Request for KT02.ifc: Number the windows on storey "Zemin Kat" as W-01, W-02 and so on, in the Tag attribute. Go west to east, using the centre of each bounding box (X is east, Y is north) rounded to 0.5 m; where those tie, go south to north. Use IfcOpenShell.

First a look at what the model holds.

```python
import ifcopenshell
import ifcopenshell.util.element
import ifcopenshell.util.placement

model = ifcopenshell.open("KT02.ifc")
print(model.schema)
storey = next(s for s in model.by_type("IfcBuildingStorey") if s.Name == "Zemin Kat")
windows = [e for e in ifcopenshell.util.element.get_decomposition(storey) if e.is_a("IfcWindow")]
for e in sorted(windows, key=lambda e: e.id()):
    origin = ifcopenshell.util.placement.get_local_placement(e.ObjectPlacement)[:3, 3]
    print(e.id(), e.Tag, e.Name, origin.round(2) + 0.0, sep=" | ")
```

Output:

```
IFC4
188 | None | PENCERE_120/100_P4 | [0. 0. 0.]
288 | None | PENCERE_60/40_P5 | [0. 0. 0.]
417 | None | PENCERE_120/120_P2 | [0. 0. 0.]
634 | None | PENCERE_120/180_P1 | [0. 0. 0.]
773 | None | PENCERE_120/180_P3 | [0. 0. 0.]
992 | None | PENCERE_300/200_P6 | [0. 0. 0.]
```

```python
import ifcopenshell
import ifcopenshell.geom
import ifcopenshell.util.element
import ifcopenshell.util.shape

model = ifcopenshell.open("KT02.ifc")
settings = ifcopenshell.geom.settings()
settings.set("use-world-coords", True)


def centre(element):
    shape = ifcopenshell.geom.create_shape(settings, element)
    return ifcopenshell.util.shape.get_bbox_centroid(shape.geometry)


storey = next(s for s in model.by_type("IfcBuildingStorey") if s.Name == "Zemin Kat")
windows = [e for e in ifcopenshell.util.element.get_decomposition(storey) if e.is_a("IfcWindow")]

# Insertion points can sit at a corner or the storey origin, so sort by the geometry (in metres).
centres = {e: centre(e) for e in windows}
windows.sort(key=lambda e: (round(centres[e][0] / 0.5), centres[e][1]))

for i, e in enumerate(windows, start=1):
    number = f"W-{i:02d}"
    e.Tag = number
    print(e.id(), number)

model.write("KT02_edited.ifc")
```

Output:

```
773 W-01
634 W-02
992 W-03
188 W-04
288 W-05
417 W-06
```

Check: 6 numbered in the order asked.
